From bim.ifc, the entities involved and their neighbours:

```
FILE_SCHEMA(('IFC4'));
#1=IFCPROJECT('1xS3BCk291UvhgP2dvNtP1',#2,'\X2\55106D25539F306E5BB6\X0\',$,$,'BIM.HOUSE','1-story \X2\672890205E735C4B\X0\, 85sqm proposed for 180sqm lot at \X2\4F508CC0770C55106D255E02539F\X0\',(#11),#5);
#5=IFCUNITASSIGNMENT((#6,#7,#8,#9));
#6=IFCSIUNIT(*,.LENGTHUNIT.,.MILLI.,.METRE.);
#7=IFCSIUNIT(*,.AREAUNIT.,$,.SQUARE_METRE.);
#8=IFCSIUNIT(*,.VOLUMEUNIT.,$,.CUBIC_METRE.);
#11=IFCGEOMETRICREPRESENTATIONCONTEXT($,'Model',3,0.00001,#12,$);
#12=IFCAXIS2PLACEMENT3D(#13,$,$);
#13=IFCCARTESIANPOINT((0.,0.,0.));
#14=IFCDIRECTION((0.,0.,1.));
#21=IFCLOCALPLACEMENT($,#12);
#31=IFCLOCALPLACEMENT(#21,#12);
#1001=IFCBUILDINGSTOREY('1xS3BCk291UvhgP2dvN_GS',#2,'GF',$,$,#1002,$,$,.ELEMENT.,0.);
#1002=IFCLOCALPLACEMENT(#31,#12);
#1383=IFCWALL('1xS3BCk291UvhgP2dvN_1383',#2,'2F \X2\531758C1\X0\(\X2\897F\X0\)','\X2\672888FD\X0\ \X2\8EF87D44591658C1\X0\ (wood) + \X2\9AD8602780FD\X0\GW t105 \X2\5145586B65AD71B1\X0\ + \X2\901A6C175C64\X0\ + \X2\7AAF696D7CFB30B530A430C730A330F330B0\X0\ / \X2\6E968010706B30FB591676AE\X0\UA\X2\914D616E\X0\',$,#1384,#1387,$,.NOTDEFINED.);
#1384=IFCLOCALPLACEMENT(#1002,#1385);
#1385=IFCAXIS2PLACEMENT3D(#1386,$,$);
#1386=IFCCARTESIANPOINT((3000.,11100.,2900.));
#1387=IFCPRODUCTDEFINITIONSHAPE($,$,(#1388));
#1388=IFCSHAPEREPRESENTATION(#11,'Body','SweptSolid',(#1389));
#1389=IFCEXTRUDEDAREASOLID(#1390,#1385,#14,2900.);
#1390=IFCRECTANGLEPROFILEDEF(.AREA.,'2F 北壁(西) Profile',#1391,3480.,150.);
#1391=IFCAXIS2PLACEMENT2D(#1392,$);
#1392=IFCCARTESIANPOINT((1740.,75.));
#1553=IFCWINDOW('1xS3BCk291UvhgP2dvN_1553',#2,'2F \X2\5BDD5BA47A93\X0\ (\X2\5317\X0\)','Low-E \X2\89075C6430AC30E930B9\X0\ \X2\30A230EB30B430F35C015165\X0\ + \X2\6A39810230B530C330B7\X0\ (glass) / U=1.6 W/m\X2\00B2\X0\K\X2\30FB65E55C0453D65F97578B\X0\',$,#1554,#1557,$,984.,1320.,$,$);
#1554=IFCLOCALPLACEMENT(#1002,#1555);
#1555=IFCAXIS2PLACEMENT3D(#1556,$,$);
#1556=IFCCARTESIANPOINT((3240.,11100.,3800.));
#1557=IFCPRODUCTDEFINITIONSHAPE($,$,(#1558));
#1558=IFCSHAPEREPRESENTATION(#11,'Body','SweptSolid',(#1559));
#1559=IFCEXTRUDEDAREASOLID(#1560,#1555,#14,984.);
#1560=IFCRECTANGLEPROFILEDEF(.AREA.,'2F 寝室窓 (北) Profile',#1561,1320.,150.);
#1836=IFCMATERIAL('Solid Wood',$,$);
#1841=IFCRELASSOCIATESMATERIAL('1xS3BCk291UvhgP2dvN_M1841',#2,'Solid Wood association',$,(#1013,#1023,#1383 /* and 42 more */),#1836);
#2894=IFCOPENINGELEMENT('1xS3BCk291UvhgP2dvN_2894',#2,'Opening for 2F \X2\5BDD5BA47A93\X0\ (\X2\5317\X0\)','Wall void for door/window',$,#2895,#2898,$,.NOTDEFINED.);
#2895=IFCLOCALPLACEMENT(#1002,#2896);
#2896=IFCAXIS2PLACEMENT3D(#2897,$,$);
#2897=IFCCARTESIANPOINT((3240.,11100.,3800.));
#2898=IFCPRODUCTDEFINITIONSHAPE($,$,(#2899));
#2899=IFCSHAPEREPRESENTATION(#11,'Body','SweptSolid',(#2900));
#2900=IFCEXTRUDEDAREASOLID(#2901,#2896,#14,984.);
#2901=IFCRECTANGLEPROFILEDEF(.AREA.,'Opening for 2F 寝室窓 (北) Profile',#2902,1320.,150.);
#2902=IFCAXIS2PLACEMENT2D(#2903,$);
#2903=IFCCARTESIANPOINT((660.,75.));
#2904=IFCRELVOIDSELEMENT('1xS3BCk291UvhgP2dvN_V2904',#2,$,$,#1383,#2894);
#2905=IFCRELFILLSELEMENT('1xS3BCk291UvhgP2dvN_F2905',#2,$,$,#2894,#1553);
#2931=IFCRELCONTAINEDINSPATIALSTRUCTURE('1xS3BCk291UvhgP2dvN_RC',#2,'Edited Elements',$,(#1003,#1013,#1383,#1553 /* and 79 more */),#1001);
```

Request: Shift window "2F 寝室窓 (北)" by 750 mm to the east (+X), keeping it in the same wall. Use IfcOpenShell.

```python
import ifcopenshell
import ifcopenshell.api.geometry
import ifcopenshell.util.placement

model = ifcopenshell.open("bim.ifc")

window = model.by_guid("1xS3BCk291UvhgP2dvN_1553")
opening = window.FillsVoids[0].RelatingOpeningElement
wall = opening.VoidsElements[0].RelatingBuildingElement

wall_matrix = ifcopenshell.util.placement.get_local_placement(wall.ObjectPlacement)
shift = wall_matrix[:3, 0] * 750.0
before = ifcopenshell.util.placement.get_local_placement(window.ObjectPlacement)[:3, 3].copy()

# The window is not placed relative to its opening, so move both.
for product in (opening, window):
    matrix = ifcopenshell.util.placement.get_local_placement(product.ObjectPlacement)
    matrix[:3, 3] += shift
    ifcopenshell.api.geometry.edit_object_placement(model, product=product, matrix=matrix, is_si=False)

after = ifcopenshell.util.placement.get_local_placement(window.ObjectPlacement)[:3, 3]
print("window moved by", (after - before).round(3) + 0.0)

model.write("bim_v2.ifc")
```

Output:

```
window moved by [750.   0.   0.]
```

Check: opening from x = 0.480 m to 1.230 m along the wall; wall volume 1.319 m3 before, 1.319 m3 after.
